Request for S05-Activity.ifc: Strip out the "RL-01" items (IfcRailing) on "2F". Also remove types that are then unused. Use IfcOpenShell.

First a look at what the model holds.

```python
import ifcopenshell
import ifcopenshell.util.element

model = ifcopenshell.open("S05-Activity.ifc")
print(model.schema)
storey = next(s for s in model.by_type("IfcBuildingStorey") if s.Name == "2F")
railings = [e for e in ifcopenshell.util.element.get_decomposition(storey) if e.is_a("IfcRailing")]
seen = {}
for e in railings:
    element_type = ifcopenshell.util.element.get_type(e)
    name = element_type.Name if element_type not in (None, e) else None
    seen[name] = seen.get(name, 0) + 1
for name, count in sorted(seen.items(), key=str):
    print(count, "x", name)
```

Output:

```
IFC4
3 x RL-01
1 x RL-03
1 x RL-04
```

```python
import ifcopenshell
import ifcopenshell.api.root
import ifcopenshell.util.element

model = ifcopenshell.open("S05-Activity.ifc")

storey = next(s for s in model.by_type("IfcBuildingStorey") if s.Name == "2F")
railings = [e for e in ifcopenshell.util.element.get_decomposition(storey) if e.is_a("IfcRailing")]
targets = [e for e in railings if (t := ifcopenshell.util.element.get_type(e)) not in (None, e) and t.Name == "RL-01"]
types = {ifcopenshell.util.element.get_type(e) for e in targets} - {None, *targets}

for e in targets:
    ifcopenshell.api.root.remove_product(model, product=e)
print(len(targets), "removed")

unused = [t for t in types if not ifcopenshell.util.element.get_types(t)]
for t in unused:
    ifcopenshell.api.root.remove_product(model, product=t)
print(len(unused), "unused types removed")

model.write("S05-Activity_edited.ifc")
```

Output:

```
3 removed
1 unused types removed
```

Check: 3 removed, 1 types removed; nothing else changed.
